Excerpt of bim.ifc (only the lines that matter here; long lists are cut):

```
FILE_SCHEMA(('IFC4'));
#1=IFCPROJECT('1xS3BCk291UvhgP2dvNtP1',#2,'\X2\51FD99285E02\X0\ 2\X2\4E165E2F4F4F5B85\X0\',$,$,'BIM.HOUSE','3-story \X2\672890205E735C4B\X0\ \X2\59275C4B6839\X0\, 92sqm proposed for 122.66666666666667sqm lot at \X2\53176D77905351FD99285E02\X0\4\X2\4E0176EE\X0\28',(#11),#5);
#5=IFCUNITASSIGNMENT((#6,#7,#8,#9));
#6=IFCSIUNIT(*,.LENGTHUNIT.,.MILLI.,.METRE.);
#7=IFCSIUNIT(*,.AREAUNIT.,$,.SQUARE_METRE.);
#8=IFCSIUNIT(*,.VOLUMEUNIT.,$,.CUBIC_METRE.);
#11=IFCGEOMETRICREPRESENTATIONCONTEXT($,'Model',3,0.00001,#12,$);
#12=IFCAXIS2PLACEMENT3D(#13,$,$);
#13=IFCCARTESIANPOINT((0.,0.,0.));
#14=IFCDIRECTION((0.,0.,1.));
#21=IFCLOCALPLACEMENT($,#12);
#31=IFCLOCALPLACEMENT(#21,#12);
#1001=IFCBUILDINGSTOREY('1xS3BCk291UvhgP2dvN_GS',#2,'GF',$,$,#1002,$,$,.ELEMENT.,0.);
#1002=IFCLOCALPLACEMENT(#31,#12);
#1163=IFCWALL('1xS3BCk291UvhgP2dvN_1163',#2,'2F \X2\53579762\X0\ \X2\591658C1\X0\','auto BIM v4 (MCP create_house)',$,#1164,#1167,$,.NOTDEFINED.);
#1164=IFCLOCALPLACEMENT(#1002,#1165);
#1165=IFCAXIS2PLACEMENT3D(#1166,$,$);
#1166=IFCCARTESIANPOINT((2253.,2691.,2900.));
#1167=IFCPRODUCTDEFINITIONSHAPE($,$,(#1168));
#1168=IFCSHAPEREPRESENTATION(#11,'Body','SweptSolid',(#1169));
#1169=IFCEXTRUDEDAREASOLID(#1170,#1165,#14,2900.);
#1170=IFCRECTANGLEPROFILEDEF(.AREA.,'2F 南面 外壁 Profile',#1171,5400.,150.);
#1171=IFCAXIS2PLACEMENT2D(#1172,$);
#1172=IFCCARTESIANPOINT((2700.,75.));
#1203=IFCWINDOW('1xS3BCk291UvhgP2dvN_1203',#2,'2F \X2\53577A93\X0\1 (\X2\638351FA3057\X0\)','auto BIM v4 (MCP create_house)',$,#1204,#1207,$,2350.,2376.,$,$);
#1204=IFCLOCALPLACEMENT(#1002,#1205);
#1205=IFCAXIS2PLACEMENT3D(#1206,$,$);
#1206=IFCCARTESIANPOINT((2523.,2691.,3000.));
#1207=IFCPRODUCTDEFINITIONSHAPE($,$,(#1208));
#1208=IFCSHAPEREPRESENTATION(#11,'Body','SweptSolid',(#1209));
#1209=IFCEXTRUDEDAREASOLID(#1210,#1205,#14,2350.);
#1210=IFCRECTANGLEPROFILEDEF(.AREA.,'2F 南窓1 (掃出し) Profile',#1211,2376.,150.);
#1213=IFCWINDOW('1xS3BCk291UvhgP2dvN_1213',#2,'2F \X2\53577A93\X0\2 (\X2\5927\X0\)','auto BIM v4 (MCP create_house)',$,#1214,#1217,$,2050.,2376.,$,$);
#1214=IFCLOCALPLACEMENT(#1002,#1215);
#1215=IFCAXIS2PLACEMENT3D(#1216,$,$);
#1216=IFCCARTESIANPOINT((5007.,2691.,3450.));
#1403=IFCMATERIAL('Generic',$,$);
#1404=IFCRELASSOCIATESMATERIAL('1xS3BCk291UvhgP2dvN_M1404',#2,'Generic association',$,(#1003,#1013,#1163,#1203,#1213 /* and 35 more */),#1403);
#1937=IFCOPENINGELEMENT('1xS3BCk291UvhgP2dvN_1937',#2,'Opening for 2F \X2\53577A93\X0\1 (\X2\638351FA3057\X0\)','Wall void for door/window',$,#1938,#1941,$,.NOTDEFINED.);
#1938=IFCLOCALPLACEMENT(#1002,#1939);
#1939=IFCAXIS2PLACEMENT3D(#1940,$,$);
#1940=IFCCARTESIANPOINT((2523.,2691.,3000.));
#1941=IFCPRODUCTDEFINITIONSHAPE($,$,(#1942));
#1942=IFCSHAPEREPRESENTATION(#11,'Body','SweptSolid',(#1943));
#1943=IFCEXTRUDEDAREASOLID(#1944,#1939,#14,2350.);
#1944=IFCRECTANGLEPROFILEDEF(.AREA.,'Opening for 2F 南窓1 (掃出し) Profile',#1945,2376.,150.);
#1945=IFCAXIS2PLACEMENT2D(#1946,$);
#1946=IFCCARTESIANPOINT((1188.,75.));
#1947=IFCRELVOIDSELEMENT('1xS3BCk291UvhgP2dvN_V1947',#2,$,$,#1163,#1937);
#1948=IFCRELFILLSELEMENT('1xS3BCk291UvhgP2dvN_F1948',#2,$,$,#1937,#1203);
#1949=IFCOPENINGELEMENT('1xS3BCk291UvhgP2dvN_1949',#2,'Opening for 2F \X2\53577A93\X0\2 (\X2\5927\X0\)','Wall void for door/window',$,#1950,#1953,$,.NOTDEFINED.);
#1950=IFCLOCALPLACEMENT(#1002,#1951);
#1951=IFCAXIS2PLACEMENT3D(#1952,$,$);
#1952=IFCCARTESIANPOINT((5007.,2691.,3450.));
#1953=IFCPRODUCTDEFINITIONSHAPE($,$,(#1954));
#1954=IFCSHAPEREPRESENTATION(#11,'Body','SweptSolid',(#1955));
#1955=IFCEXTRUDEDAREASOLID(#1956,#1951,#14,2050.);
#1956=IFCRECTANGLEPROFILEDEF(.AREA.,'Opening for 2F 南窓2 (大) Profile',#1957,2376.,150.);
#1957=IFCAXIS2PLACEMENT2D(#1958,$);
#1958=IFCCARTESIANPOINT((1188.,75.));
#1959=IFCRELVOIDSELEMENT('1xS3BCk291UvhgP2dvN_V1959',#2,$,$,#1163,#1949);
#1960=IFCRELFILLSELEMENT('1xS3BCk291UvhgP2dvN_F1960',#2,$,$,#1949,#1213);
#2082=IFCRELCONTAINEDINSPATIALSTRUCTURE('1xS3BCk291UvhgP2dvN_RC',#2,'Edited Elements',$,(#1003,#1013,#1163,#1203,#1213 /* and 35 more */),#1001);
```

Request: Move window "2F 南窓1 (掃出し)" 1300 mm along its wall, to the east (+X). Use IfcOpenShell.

```python
import ifcopenshell
import ifcopenshell.api.geometry
import ifcopenshell.util.placement

model = ifcopenshell.open("bim.ifc")

window = model.by_guid("1xS3BCk291UvhgP2dvN_1203")
opening = window.FillsVoids[0].RelatingOpeningElement
wall = opening.VoidsElements[0].RelatingBuildingElement

wall_matrix = ifcopenshell.util.placement.get_local_placement(wall.ObjectPlacement)
shift = wall_matrix[:3, 0] * 1300.0
before = ifcopenshell.util.placement.get_local_placement(window.ObjectPlacement)[:3, 3].copy()

# The window is not placed relative to its opening, so move both.
for product in (opening, window):
    matrix = ifcopenshell.util.placement.get_local_placement(product.ObjectPlacement)
    matrix[:3, 3] += shift
    ifcopenshell.api.geometry.edit_object_placement(model, product=product, matrix=matrix, is_si=False)

after = ifcopenshell.util.placement.get_local_placement(window.ObjectPlacement)[:3, 3]
print("window moved by", (after - before).round(3) + 0.0)

model.write("bim_v2.ifc")
```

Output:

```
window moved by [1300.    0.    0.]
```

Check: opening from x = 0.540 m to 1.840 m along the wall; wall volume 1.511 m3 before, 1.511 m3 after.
